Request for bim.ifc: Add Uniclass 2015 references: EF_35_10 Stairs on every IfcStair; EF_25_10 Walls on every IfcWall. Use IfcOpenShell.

First a look at what the model holds.

```python
import ifcopenshell

model = ifcopenshell.open("bim.ifc")
print(model.schema)
print("classifications:", [c.Name for c in model.by_type("IfcClassification")])
for ifc_class in ("IfcDoor", "IfcRoof", "IfcStair", "IfcWall", "IfcWindow"):
    print(ifc_class, len(model.by_type(ifc_class)))
```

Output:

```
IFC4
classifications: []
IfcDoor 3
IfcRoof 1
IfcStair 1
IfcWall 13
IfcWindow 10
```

```python
import ifcopenshell
import ifcopenshell.api.classification

model = ifcopenshell.open("bim.ifc")

system = ifcopenshell.api.classification.add_classification(model, classification="Uniclass 2015")

codes = {
    "IfcStair": ("EF_35_10", "Stairs"),
    "IfcWall": ("EF_25_10", "Walls"),
}
for ifc_class, (code, name) in codes.items():
    products = model.by_type(ifc_class)
    ifcopenshell.api.classification.add_reference(
        model, products=products, classification=system, identification=code, name=name
    )
    print(code, len(products))

model.write("bim-out.ifc")
```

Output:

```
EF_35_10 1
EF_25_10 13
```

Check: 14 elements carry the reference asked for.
